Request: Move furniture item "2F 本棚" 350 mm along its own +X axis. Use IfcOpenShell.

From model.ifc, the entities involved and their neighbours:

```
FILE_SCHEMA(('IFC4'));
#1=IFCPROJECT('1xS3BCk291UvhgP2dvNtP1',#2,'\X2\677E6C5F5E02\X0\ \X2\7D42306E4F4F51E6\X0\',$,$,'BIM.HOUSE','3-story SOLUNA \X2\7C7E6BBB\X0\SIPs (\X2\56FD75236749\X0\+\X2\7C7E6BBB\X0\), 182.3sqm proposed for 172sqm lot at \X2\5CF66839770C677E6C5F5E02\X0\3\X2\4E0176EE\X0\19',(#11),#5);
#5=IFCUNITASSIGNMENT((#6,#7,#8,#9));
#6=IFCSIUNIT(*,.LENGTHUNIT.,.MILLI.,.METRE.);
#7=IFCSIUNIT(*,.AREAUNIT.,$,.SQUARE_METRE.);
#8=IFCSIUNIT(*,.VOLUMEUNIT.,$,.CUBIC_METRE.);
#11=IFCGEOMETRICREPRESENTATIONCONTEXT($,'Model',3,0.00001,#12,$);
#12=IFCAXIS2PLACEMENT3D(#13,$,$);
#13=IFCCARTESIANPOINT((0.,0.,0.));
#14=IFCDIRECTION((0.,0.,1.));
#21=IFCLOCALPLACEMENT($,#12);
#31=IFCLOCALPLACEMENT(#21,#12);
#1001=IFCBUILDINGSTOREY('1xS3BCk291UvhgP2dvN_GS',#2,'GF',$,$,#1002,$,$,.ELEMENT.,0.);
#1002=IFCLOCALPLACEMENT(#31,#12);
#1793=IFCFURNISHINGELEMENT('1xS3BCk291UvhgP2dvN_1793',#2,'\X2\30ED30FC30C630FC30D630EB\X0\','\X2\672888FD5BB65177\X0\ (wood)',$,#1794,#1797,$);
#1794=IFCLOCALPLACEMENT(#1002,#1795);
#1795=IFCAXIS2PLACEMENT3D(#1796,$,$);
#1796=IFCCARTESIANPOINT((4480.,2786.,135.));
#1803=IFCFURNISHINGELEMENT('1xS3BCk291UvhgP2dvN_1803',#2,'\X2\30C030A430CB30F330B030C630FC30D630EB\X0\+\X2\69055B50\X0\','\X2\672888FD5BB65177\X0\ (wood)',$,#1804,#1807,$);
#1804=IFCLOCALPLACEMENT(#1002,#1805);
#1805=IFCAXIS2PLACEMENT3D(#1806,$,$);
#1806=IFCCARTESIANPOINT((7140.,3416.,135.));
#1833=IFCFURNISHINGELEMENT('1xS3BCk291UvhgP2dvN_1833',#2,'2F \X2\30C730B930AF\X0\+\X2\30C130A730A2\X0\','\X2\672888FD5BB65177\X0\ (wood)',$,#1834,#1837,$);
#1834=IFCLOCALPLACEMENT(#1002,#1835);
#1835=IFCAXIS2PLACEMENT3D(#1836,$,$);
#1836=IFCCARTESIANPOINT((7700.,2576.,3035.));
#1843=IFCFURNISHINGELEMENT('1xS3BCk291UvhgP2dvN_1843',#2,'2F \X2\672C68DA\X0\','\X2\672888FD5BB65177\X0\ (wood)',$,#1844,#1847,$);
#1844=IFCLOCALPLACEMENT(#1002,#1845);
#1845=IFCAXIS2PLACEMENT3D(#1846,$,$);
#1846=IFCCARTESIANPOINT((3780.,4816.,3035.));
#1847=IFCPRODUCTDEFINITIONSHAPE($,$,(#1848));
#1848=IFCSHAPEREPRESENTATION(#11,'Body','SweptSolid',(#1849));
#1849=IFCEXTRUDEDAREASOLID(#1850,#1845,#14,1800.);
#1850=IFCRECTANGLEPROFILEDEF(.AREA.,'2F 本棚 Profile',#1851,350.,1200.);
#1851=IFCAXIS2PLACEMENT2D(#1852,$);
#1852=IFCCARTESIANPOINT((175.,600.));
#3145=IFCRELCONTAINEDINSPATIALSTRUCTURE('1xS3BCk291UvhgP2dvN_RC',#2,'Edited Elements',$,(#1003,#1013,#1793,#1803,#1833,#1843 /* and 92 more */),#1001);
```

```python
import ifcopenshell
import ifcopenshell.api.geometry
import ifcopenshell.util.placement

model = ifcopenshell.open("model.ifc")

item = model.by_id(1843)
matrix = ifcopenshell.util.placement.get_local_placement(item.ObjectPlacement)
matrix[:3, 3] += matrix[:3, 0] * 350.0
ifcopenshell.api.geometry.edit_object_placement(model, product=item, matrix=matrix, is_si=False)

print(ifcopenshell.util.placement.get_local_placement(item.ObjectPlacement).round(3) + 0.0)

model.write("model_rev.ifc")
```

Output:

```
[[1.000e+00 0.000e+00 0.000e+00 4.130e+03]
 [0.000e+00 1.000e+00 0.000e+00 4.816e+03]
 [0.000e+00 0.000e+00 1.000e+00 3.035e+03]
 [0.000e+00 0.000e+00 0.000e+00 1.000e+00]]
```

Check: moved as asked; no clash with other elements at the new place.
